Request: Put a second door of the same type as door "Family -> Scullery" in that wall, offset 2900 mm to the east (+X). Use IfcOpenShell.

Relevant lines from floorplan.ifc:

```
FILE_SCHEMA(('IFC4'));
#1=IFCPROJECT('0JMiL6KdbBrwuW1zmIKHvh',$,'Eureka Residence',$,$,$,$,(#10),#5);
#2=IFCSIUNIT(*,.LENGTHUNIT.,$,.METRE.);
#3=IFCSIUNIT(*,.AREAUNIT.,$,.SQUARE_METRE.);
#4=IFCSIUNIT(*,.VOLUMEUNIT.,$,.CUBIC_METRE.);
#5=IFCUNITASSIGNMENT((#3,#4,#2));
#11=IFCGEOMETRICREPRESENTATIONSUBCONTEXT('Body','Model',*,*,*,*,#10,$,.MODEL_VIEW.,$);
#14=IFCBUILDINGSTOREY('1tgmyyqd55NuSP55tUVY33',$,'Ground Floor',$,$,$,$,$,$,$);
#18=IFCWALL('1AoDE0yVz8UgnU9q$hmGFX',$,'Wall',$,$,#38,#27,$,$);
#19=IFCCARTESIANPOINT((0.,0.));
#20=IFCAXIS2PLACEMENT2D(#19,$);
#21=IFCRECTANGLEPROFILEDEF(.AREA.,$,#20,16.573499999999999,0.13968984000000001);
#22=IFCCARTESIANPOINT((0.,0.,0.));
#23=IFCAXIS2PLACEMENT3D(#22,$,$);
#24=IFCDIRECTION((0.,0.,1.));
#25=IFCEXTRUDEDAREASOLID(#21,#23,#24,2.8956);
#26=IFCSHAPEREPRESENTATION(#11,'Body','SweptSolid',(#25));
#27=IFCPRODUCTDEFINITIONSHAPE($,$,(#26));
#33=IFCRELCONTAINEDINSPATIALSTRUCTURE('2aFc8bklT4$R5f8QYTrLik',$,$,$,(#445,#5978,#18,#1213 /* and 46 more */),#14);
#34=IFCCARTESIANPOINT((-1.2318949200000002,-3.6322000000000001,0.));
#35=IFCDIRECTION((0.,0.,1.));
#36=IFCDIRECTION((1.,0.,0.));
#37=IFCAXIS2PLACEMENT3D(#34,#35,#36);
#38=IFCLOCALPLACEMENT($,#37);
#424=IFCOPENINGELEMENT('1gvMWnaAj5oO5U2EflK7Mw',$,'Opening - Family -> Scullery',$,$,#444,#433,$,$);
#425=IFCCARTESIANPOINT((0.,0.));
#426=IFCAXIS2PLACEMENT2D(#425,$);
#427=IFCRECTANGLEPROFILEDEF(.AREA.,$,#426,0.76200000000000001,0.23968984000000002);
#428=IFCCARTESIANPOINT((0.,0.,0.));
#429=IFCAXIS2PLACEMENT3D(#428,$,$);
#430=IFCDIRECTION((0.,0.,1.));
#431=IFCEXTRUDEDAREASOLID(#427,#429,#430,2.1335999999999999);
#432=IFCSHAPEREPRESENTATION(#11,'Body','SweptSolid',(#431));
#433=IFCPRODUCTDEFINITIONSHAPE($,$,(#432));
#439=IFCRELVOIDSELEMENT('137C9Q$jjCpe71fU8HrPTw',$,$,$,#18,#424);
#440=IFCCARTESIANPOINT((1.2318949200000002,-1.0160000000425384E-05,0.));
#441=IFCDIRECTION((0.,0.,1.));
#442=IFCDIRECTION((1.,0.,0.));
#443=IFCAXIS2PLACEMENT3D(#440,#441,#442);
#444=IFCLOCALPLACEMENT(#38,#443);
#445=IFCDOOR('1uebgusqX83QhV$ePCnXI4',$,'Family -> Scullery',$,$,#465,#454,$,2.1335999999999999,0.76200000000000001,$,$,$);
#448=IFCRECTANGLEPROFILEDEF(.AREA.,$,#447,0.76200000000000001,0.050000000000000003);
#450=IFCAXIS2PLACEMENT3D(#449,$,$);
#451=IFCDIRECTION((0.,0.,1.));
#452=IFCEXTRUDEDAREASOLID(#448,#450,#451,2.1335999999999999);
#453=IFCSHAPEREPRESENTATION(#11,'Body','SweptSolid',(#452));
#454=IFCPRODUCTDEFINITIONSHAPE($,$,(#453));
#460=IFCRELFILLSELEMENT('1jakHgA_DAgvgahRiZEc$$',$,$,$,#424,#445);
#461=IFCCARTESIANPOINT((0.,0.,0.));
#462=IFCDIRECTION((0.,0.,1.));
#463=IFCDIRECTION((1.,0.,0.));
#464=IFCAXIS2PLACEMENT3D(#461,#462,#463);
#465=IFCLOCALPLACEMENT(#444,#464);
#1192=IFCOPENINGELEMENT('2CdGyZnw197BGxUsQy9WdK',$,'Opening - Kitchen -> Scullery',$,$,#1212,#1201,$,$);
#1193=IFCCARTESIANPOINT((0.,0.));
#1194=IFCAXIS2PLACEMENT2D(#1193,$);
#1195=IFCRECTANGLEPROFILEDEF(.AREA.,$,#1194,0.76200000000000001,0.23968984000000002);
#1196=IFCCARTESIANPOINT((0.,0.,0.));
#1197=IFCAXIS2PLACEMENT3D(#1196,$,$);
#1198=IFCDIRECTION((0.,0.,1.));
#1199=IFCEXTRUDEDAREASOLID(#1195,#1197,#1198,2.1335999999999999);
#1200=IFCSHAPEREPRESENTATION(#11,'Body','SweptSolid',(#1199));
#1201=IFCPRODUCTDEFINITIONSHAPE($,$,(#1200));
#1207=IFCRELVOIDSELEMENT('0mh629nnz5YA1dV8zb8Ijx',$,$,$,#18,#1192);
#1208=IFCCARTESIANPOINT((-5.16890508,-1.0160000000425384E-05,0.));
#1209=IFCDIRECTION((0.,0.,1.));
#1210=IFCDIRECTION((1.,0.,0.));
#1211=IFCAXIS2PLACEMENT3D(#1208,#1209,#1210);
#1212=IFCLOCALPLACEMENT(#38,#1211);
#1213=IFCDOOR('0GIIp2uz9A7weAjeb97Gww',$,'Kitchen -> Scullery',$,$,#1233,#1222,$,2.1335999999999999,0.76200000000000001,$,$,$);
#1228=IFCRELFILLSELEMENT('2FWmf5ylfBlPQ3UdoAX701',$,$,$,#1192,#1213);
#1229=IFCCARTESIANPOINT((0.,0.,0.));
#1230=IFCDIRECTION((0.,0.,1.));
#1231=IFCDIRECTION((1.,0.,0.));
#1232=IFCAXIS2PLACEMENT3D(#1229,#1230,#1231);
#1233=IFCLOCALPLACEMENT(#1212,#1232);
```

```python
import ifcopenshell
import ifcopenshell.api.feature
import ifcopenshell.api.geometry
import ifcopenshell.api.root
import ifcopenshell.geom
import ifcopenshell.util.element
import ifcopenshell.util.placement
import ifcopenshell.util.shape
import ifcopenshell.util.unit

model = ifcopenshell.open("floorplan.ifc")
unit_scale = ifcopenshell.util.unit.calculate_unit_scale(model)
settings = ifcopenshell.geom.settings()


def volume(element):
    """Net volume in cubic metres, openings subtracted."""
    shape = ifcopenshell.geom.create_shape(settings, element)
    return ifcopenshell.util.shape.get_volume(shape.geometry)


door = model.by_guid("1uebgusqX83QhV$ePCnXI4")
opening = door.FillsVoids[0].RelatingOpeningElement
wall = opening.VoidsElements[0].RelatingBuildingElement
before = volume(wall)
shift = ifcopenshell.util.placement.get_local_placement(wall.ObjectPlacement)[:3, 0] * 2.9 / unit_scale

# copy_class copies the void relationship, type, container and properties, but no geometry.
new_opening = ifcopenshell.api.root.copy_class(model, product=opening)
new_opening.Representation = ifcopenshell.util.element.copy_deep(
    model, opening.Representation, exclude=["IfcGeometricRepresentationContext", "IfcRepresentationMap"]
)
new_door = ifcopenshell.api.root.copy_class(model, product=door)
new_door.Representation = ifcopenshell.util.element.copy_deep(
    model, door.Representation, exclude=["IfcGeometricRepresentationContext", "IfcRepresentationMap"]
)
ifcopenshell.api.feature.add_filling(model, opening=new_opening, element=new_door)

for old, new in ((opening, new_opening), (door, new_door)):
    matrix = ifcopenshell.util.placement.get_local_placement(old.ObjectPlacement)
    matrix[:3, 3] += shift
    ifcopenshell.api.geometry.edit_object_placement(model, product=new, matrix=matrix, is_si=False)

after = volume(wall)

print(f"wall volume {before:.3f} -> {after:.3f} m3")

model.write("floorplan_rev.ifc")
```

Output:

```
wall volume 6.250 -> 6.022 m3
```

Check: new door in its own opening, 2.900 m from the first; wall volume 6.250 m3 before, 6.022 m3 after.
